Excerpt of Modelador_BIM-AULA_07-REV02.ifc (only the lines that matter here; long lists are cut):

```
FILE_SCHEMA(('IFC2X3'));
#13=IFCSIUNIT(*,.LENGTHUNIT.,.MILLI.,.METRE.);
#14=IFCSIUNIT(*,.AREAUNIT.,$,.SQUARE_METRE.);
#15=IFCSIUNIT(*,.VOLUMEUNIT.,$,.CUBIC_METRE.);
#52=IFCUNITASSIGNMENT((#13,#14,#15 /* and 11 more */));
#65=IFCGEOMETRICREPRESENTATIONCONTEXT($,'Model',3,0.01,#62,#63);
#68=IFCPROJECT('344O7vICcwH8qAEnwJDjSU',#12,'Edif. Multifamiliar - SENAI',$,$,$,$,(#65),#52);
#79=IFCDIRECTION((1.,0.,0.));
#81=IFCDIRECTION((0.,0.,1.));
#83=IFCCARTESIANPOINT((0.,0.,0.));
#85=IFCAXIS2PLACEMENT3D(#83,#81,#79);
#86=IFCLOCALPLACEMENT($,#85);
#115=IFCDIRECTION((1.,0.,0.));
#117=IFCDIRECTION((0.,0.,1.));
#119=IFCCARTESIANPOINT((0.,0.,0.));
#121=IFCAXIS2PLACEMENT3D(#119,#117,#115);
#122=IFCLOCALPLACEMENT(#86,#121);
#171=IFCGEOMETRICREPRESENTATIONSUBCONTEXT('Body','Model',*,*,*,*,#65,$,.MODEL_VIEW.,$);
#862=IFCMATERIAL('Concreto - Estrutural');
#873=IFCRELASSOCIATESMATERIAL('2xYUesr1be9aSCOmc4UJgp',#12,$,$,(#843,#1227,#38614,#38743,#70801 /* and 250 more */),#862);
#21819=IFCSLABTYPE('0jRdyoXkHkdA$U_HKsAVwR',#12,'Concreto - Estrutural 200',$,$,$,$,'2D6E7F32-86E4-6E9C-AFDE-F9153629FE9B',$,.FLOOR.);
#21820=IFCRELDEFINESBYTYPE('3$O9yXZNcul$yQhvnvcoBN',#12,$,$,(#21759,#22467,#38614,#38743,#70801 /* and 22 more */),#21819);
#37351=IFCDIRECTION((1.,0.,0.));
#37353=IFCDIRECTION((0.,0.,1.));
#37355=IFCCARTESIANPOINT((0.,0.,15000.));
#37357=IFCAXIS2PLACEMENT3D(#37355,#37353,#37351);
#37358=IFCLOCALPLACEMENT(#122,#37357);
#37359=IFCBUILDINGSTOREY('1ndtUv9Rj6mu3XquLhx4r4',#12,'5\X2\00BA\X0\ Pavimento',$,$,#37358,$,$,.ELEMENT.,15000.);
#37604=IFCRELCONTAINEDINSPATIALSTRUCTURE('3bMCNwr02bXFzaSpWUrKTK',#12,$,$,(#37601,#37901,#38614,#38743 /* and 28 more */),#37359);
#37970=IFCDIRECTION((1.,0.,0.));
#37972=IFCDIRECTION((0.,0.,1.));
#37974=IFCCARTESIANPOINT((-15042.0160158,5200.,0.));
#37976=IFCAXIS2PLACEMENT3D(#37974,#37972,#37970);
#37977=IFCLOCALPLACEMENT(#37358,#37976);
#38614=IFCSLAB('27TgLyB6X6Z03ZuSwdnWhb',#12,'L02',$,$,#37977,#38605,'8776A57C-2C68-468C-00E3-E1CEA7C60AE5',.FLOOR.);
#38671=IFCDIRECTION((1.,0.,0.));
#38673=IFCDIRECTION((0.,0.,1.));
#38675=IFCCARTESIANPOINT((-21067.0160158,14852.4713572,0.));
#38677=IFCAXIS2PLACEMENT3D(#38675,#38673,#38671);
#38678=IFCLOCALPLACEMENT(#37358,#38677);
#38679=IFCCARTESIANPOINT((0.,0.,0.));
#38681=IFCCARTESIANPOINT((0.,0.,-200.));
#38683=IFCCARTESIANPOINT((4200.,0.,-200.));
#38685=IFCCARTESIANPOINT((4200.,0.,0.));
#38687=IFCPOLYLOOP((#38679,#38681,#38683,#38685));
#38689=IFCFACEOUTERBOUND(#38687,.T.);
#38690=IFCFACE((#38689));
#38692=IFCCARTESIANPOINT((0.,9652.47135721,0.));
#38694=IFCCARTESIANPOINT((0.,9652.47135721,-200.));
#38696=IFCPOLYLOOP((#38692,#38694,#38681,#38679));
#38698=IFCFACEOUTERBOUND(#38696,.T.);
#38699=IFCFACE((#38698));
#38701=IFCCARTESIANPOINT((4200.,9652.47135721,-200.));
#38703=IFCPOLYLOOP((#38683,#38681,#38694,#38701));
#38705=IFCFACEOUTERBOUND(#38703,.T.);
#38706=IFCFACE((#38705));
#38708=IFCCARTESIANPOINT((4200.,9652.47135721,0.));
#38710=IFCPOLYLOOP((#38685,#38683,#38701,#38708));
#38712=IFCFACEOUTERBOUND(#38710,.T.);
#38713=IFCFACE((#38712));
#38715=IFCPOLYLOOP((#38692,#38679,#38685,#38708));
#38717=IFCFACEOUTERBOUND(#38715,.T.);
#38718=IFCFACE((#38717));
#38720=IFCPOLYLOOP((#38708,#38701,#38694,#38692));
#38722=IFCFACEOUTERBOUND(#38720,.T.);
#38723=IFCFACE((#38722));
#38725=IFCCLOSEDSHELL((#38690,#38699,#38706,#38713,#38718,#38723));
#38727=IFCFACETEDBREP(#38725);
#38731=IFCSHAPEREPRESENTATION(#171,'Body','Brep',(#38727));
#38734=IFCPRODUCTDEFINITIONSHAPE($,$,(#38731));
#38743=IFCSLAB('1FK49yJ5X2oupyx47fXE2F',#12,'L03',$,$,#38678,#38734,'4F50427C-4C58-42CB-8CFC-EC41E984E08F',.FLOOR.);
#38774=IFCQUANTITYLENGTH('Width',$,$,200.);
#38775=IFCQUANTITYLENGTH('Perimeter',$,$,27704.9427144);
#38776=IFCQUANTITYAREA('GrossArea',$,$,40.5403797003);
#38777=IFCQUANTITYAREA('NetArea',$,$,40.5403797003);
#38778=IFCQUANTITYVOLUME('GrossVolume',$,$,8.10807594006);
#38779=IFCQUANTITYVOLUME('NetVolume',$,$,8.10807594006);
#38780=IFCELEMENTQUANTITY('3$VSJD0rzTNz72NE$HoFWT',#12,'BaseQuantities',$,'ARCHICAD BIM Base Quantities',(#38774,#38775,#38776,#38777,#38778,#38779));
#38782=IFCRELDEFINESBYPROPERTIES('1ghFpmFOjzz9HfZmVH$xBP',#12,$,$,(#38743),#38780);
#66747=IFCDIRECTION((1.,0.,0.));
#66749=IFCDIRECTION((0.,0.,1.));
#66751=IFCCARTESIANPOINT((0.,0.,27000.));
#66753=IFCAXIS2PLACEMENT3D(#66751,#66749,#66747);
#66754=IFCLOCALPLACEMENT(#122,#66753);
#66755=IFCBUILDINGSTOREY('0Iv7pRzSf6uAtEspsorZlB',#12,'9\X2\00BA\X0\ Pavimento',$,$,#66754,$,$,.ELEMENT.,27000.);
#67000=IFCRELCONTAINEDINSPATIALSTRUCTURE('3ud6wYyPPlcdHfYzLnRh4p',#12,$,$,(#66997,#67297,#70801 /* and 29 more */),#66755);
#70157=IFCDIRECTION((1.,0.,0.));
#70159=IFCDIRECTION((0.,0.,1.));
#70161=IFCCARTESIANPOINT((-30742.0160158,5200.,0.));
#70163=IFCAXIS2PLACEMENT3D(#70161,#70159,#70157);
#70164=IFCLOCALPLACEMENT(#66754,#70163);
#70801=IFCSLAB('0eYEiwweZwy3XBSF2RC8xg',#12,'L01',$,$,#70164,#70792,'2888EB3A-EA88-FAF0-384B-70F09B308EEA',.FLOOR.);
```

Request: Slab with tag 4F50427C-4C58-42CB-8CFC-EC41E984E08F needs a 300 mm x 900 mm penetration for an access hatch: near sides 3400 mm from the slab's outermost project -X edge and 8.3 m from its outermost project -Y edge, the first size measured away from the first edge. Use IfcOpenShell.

```python
import numpy as np
import ifcopenshell
import ifcopenshell.api.feature
import ifcopenshell.api.geometry
import ifcopenshell.api.pset
import ifcopenshell.api.root
import ifcopenshell.geom
import ifcopenshell.util.element
import ifcopenshell.util.placement
import ifcopenshell.util.representation
import ifcopenshell.util.shape
import ifcopenshell.util.unit

model = ifcopenshell.open("Modelador_BIM-AULA_07-REV02.ifc")
unit_scale = ifcopenshell.util.unit.calculate_unit_scale(model)
area_scale = ifcopenshell.util.unit.calculate_unit_scale(model, "AREAUNIT")
volume_scale = ifcopenshell.util.unit.calculate_unit_scale(model, "VOLUMEUNIT")
settings = ifcopenshell.geom.settings()


def volume(element):
    """Net volume in cubic metres, openings subtracted."""
    shape = ifcopenshell.geom.create_shape(settings, element)
    return ifcopenshell.util.shape.get_volume(shape.geometry)


slab = model.by_guid("1FK49yJ5X2oupyx47fXE2F")
before = volume(slab)

# Extent in the slab's own axes, in metres. The edges named are its -X and -Y sides.
slab_shape = ifcopenshell.geom.create_shape(settings, slab)
vertices = ifcopenshell.util.shape.get_vertices(slab_shape.geometry)
x_min, y_min, bottom = vertices.min(axis=0)
top = vertices[:, 2].max()

opening = ifcopenshell.api.root.create_entity(model, ifc_class="IfcOpeningElement", name="Access hatch opening")
context = ifcopenshell.util.representation.get_context(model, "Model", "Body", "MODEL_VIEW")
width, depth = 0.3, 0.9
outline = [(0.0, 0.0), (width, 0.0), (width, depth), (0.0, depth), (0.0, 0.0)]
# Overshoot both faces by 50 mm so the cut is clean.
shape = ifcopenshell.api.geometry.add_slab_representation(
    model, context=context, depth=top - bottom + 0.1, polyline=outline
)
ifcopenshell.api.geometry.assign_representation(model, product=opening, representation=shape)

matrix = ifcopenshell.util.placement.get_local_placement(slab.ObjectPlacement)
matrix[:, 3] = matrix @ np.append(np.array([x_min + 3.4, y_min + 8.3, bottom - 0.05]) / unit_scale, 1.0)
ifcopenshell.api.geometry.edit_object_placement(model, product=opening, matrix=matrix, is_si=False)
ifcopenshell.api.feature.add_feature(model, feature=opening, element=slab)

after = volume(slab)

# Update the slab's stored quantities.
qto = model.by_id(ifcopenshell.util.element.get_pset(slab, "BaseQuantities", should_inherit=False)["id"])
ifcopenshell.api.pset.edit_qto(model, qto=qto, properties={
    "NetArea": after / (top - bottom) / area_scale,
    "NetVolume": after / volume_scale,
})

print(f"slab volume {before:.3f} -> {after:.3f} m3")

model.write("Modelador_BIM-AULA_07-REV02_rev.ifc")
```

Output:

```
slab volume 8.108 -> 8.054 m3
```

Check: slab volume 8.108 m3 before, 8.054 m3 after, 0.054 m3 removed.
